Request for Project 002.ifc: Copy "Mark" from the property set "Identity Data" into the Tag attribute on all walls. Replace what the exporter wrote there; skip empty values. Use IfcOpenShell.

First a look at what the model holds.

```python
import ifcopenshell
import ifcopenshell.util.element

model = ifcopenshell.open("Project 002.ifc")
print(model.schema)
walls = model.by_type("IfcWall")
print(len(walls), "walls")
for e in walls[:8]:
    source = ifcopenshell.util.element.get_pset(e, "Identity Data", "Mark")
    target = e.Tag
    print(e.id(), repr(source), repr(target), sep=" | ")
```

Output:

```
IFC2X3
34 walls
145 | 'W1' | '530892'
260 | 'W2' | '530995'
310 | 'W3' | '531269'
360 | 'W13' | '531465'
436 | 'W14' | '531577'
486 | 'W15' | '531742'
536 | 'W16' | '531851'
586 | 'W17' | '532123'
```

```python
import ifcopenshell
import ifcopenshell.util.element

model = ifcopenshell.open("Project 002.ifc")

count = 0
for e in model.by_type("IfcWall"):
    value = ifcopenshell.util.element.get_pset(e, "Identity Data", "Mark")
    current = e.Tag
    if not value or not value.strip() or current == value:
        continue
    e.Tag = value
    count += 1

print(count, "walls updated")

model.write("Project 002_v2.ifc")
```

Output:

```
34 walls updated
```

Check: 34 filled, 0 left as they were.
